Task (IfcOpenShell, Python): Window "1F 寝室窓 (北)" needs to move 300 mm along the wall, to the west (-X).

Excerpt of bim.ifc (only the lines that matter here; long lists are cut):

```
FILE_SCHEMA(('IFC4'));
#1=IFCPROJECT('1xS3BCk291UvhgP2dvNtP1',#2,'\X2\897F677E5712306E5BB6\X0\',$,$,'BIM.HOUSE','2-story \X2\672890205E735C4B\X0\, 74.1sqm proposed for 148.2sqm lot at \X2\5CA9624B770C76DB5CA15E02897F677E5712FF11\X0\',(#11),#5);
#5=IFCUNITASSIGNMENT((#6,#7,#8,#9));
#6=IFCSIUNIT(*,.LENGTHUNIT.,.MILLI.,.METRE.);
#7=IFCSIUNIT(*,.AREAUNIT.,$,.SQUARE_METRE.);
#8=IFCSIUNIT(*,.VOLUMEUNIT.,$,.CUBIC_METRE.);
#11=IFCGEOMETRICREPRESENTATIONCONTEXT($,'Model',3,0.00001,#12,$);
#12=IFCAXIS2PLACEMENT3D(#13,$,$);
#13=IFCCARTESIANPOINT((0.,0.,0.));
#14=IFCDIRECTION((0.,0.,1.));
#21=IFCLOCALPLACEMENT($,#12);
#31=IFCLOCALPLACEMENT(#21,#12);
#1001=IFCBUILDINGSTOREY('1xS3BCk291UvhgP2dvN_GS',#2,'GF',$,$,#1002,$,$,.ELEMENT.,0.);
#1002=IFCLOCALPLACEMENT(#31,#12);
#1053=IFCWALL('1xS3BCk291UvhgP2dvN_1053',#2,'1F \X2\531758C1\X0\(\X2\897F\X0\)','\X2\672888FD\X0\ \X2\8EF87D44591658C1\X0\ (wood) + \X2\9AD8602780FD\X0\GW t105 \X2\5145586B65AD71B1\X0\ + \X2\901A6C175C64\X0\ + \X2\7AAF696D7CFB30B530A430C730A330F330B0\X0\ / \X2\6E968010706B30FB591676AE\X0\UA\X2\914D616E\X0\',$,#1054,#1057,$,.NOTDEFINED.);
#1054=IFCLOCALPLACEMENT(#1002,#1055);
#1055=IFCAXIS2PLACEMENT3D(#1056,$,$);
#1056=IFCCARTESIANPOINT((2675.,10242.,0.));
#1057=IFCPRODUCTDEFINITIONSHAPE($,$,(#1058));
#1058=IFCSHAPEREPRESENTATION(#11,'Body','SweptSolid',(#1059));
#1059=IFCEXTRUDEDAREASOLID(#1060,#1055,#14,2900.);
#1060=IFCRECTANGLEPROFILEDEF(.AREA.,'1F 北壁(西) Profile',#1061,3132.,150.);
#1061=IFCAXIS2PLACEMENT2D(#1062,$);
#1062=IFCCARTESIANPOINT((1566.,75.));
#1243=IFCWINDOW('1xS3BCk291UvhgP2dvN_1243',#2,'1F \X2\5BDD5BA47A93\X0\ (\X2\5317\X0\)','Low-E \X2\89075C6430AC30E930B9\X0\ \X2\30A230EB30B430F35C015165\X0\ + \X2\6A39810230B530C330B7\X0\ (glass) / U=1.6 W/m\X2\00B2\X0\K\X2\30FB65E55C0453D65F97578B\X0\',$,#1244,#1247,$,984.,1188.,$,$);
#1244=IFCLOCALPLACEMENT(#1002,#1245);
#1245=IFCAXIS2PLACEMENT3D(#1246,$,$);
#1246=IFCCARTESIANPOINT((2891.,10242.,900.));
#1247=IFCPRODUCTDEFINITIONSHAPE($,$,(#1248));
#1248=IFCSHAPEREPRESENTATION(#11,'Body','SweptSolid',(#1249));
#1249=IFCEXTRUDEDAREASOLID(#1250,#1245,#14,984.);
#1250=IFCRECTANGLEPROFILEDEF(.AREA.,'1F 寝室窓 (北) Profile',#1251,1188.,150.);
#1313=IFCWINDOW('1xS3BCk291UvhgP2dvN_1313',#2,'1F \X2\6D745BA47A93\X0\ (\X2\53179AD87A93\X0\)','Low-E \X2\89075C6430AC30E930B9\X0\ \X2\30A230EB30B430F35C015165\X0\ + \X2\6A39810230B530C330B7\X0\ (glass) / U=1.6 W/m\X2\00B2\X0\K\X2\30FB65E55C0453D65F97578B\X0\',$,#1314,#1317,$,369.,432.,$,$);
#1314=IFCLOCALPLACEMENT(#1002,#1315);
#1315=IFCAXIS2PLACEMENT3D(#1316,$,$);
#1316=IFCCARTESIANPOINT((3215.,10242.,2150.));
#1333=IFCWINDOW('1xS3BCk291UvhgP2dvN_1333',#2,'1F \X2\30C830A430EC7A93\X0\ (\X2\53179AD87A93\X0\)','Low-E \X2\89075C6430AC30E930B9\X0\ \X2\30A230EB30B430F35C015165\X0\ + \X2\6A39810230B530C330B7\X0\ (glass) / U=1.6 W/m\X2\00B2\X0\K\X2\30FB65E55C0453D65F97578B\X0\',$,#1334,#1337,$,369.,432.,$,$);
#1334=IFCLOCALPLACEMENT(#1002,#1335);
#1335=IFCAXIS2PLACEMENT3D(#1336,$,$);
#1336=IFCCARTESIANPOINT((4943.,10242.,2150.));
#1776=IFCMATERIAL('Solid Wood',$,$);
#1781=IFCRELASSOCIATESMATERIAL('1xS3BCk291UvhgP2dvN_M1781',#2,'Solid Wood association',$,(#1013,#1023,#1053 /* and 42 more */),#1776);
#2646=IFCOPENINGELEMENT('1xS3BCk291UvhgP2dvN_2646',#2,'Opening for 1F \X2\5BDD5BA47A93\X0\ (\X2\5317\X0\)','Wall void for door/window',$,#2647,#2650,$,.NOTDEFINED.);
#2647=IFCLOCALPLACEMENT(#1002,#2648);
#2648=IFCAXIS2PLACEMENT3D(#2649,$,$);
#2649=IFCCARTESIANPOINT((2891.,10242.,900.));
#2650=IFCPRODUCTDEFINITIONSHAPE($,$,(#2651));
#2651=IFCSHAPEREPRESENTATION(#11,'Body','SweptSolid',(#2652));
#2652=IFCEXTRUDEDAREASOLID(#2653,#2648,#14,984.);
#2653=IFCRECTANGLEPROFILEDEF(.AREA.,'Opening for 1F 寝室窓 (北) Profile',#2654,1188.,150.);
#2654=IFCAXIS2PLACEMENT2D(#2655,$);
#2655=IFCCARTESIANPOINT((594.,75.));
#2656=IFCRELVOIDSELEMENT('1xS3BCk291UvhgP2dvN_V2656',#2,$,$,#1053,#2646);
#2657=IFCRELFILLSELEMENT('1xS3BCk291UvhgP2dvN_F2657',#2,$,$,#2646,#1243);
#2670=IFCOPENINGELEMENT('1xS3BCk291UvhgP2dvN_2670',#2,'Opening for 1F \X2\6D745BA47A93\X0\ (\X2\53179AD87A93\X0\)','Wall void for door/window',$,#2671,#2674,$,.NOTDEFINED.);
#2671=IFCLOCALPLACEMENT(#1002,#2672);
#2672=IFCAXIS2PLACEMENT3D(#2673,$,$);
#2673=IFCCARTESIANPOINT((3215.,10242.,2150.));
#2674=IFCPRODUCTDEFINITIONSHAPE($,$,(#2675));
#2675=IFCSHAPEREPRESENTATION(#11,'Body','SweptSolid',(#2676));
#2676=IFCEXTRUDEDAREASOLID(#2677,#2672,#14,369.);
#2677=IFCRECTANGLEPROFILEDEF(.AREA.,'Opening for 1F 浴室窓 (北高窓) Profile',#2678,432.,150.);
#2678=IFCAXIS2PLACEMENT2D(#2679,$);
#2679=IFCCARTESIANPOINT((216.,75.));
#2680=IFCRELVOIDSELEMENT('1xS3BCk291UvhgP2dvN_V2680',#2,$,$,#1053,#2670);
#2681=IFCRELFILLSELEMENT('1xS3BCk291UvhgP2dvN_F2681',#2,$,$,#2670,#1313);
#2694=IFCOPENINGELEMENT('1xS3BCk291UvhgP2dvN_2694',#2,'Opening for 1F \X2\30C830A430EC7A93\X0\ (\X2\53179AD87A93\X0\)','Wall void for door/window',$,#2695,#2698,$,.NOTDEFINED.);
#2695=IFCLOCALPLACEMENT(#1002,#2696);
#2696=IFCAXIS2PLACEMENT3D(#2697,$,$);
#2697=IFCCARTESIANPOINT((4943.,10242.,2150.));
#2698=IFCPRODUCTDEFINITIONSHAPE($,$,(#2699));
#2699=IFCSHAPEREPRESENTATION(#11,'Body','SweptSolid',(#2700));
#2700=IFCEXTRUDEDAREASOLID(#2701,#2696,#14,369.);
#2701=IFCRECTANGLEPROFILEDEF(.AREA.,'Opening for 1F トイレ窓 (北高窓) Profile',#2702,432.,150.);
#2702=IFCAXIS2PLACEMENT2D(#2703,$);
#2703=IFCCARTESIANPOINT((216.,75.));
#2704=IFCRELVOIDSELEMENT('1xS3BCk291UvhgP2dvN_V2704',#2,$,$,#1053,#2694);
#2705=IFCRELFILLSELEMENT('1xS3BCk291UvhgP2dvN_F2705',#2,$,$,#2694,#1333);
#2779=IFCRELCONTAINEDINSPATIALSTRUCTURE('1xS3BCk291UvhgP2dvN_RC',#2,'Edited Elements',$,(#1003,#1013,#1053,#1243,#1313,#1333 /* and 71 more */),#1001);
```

```python
import ifcopenshell
import ifcopenshell.api.geometry
import ifcopenshell.util.placement

model = ifcopenshell.open("bim.ifc")

window = model.by_guid("1xS3BCk291UvhgP2dvN_1243")
opening = window.FillsVoids[0].RelatingOpeningElement
wall = opening.VoidsElements[0].RelatingBuildingElement

wall_matrix = ifcopenshell.util.placement.get_local_placement(wall.ObjectPlacement)
shift = wall_matrix[:3, 0] * -300.0
before = ifcopenshell.util.placement.get_local_placement(window.ObjectPlacement)[:3, 3].copy()

# The window is not placed relative to its opening, so move both.
for product in (opening, window):
    matrix = ifcopenshell.util.placement.get_local_placement(product.ObjectPlacement)
    matrix[:3, 3] += shift
    ifcopenshell.api.geometry.edit_object_placement(model, product=product, matrix=matrix, is_si=False)

after = ifcopenshell.util.placement.get_local_placement(window.ObjectPlacement)[:3, 3]
print("window moved by", (after - before).round(3) + 0.0)

model.write("bim_edited.ifc")
```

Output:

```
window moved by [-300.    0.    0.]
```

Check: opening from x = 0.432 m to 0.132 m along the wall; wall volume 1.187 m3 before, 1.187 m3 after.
